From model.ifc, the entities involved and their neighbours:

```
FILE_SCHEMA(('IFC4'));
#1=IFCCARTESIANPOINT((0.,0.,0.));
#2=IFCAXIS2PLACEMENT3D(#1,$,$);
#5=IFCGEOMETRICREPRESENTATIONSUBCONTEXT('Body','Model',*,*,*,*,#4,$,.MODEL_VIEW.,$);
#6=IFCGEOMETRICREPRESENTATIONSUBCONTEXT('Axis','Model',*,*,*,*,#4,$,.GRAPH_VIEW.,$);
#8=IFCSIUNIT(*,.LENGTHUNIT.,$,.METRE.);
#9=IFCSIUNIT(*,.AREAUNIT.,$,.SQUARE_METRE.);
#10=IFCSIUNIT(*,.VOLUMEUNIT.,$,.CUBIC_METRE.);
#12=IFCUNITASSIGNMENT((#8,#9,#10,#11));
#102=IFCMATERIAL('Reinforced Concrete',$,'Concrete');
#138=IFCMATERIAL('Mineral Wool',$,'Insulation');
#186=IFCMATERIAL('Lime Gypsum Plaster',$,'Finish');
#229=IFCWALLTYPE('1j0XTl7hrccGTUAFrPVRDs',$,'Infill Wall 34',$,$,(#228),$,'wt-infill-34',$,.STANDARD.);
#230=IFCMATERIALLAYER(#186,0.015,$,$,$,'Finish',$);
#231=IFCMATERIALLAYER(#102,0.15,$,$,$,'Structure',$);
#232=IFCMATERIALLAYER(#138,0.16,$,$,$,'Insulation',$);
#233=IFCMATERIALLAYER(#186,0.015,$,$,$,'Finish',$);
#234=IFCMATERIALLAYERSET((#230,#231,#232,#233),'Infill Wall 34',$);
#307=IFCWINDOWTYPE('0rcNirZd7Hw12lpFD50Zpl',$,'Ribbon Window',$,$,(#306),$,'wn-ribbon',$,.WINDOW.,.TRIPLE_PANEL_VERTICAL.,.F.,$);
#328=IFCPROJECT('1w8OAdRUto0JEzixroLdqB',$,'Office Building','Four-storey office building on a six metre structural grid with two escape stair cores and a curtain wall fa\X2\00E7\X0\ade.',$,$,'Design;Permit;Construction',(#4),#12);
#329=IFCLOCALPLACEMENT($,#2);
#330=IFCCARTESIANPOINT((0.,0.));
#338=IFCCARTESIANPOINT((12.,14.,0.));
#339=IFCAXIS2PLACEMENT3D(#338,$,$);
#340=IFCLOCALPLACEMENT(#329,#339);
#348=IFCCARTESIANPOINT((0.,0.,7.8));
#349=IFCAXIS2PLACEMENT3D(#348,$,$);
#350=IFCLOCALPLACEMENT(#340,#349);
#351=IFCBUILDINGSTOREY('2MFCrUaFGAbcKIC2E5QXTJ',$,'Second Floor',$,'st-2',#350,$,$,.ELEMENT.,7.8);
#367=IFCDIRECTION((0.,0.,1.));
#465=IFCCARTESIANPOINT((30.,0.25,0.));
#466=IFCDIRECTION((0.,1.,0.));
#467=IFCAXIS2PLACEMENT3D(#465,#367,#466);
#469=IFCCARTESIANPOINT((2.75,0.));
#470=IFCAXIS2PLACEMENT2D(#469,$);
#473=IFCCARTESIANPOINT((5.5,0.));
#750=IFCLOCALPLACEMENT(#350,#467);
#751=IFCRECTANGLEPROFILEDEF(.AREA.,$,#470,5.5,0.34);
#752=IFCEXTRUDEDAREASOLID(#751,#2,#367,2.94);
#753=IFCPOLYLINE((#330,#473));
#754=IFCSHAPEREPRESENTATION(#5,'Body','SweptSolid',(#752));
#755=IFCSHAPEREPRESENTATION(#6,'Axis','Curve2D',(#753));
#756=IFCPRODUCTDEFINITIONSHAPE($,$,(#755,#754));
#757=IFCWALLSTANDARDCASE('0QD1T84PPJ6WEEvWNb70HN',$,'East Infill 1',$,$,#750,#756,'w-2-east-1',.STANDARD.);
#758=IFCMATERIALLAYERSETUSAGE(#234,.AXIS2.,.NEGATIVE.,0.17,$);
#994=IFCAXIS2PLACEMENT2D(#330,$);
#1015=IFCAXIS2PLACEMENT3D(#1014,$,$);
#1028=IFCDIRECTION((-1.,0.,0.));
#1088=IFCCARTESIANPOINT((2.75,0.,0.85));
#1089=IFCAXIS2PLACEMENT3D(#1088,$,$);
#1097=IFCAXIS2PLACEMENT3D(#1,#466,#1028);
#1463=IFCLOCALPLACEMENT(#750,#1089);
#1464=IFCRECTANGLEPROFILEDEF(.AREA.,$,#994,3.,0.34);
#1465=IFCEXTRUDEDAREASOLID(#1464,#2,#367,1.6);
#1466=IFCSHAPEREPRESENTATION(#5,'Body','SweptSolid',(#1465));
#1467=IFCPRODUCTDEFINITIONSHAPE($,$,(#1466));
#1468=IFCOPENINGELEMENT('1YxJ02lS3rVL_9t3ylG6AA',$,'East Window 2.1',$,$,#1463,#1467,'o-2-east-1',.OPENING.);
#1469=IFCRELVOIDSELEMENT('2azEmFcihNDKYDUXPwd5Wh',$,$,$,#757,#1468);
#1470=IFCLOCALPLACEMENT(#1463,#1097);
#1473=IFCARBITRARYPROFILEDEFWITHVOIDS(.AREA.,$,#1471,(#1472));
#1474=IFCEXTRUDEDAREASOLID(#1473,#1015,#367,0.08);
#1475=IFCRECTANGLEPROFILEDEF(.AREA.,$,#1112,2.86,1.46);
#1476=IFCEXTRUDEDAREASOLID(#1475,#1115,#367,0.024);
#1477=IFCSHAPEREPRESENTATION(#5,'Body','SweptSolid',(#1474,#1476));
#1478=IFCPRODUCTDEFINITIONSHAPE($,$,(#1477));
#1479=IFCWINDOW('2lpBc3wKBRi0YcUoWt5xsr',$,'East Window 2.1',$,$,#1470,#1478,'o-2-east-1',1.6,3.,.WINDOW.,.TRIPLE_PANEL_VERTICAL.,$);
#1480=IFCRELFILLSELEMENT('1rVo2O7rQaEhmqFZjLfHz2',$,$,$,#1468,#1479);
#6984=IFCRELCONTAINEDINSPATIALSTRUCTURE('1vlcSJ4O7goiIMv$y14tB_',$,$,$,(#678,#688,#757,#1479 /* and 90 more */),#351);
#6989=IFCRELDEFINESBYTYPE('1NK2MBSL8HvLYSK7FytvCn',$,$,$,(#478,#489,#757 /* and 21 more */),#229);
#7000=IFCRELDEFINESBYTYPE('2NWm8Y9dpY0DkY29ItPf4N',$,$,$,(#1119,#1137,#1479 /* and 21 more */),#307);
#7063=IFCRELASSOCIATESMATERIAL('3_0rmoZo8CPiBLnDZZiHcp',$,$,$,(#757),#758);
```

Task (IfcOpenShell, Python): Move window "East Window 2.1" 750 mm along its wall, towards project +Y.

```python
import ifcopenshell
import ifcopenshell.api.geometry
import ifcopenshell.util.placement

model = ifcopenshell.open("model.ifc")

window = model.by_id(1479)
opening = window.FillsVoids[0].RelatingOpeningElement
wall = opening.VoidsElements[0].RelatingBuildingElement

wall_matrix = ifcopenshell.util.placement.get_local_placement(wall.ObjectPlacement)
shift = wall_matrix[:3, 0] * 0.75
before = ifcopenshell.util.placement.get_local_placement(window.ObjectPlacement)[:3, 3].copy()

# The window is placed relative to its opening, so it follows when the opening moves.
matrix = ifcopenshell.util.placement.get_local_placement(opening.ObjectPlacement)
matrix[:3, 3] += shift
ifcopenshell.api.geometry.edit_object_placement(
    model, product=opening, matrix=matrix, is_si=False, should_transform_children=True
)

after = ifcopenshell.util.placement.get_local_placement(window.ObjectPlacement)[:3, 3]
print("window moved by", (after - before).round(3) + 0.0)

model.write("model_updated.ifc")
```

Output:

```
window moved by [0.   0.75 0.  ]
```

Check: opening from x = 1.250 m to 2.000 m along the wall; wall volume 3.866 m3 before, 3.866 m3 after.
